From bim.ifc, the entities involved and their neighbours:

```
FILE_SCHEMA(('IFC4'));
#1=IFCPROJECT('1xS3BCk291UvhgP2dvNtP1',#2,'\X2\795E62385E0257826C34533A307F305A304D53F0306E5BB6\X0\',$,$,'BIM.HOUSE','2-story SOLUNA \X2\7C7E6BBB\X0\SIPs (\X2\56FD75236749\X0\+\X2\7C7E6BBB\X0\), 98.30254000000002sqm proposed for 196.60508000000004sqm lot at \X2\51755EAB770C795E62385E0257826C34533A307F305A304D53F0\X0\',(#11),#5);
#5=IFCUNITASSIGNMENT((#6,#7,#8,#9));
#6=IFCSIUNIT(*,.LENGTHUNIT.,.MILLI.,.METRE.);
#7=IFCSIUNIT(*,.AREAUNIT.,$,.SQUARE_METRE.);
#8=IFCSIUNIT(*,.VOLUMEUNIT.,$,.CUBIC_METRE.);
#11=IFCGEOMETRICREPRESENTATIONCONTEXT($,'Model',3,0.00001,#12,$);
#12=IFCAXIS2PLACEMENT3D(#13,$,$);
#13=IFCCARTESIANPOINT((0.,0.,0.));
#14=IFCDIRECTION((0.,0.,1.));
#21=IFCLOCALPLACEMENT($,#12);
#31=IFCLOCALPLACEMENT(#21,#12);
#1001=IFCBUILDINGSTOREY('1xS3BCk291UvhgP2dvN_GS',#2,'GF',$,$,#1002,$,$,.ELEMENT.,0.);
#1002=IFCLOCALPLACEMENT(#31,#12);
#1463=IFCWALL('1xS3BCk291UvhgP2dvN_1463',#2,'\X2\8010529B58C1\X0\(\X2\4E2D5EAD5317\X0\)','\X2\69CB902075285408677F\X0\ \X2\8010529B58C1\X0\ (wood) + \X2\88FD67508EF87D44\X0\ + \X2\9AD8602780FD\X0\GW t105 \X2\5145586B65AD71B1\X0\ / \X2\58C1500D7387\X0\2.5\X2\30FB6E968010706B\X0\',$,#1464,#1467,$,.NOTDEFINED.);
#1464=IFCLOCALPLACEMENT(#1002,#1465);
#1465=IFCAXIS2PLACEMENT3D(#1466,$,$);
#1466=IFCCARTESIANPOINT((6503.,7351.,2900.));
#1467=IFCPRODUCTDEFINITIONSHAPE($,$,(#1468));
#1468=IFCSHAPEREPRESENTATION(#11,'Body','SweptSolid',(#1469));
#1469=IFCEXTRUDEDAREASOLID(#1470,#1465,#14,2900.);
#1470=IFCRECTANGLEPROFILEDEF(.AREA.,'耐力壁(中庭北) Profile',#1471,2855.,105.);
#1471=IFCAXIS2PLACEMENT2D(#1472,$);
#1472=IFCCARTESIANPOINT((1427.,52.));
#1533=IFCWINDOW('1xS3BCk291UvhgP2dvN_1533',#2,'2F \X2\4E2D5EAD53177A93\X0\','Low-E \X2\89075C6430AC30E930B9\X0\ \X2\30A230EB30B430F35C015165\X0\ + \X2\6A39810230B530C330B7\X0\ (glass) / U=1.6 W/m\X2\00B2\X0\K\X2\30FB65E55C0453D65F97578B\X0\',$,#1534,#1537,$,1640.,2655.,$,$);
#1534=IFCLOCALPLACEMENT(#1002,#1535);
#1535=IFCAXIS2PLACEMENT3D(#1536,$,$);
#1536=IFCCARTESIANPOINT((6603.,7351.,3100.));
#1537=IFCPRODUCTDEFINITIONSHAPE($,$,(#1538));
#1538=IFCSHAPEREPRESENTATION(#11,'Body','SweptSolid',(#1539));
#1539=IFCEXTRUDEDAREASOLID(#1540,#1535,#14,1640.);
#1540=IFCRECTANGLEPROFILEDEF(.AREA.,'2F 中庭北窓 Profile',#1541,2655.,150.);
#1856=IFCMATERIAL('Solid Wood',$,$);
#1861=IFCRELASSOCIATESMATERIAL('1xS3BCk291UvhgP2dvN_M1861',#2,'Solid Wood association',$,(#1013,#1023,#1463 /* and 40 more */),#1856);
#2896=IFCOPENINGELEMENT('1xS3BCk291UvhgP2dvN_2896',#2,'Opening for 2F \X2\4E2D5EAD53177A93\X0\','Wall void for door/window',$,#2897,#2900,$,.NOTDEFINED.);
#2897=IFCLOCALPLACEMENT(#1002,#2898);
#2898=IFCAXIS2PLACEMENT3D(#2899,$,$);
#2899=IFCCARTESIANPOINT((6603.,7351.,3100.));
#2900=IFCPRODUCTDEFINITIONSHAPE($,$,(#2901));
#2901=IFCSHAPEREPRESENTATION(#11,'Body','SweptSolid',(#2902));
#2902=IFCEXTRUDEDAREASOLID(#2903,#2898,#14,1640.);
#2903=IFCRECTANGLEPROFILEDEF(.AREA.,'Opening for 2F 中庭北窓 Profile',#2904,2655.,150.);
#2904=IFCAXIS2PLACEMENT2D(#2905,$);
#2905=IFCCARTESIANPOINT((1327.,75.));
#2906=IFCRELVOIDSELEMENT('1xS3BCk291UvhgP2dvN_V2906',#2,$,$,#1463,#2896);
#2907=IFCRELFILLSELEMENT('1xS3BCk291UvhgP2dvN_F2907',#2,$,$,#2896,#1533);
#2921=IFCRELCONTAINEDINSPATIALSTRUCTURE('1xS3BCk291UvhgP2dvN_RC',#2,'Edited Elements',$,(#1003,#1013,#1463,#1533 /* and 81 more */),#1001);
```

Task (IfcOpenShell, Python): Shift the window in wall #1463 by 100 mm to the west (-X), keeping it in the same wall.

```python
import ifcopenshell
import ifcopenshell.api.geometry
import ifcopenshell.util.placement
import ifcopenshell.util.unit

model = ifcopenshell.open("bim.ifc")
unit_scale = ifcopenshell.util.unit.calculate_unit_scale(model)

window = model.by_id(1533)
opening = window.FillsVoids[0].RelatingOpeningElement
wall = opening.VoidsElements[0].RelatingBuildingElement

wall_matrix = ifcopenshell.util.placement.get_local_placement(wall.ObjectPlacement)
shift = wall_matrix[:3, 0] * -0.1 / unit_scale
before = ifcopenshell.util.placement.get_local_placement(window.ObjectPlacement)[:3, 3].copy()

# The window is not placed relative to its opening, so move both.
for product in (opening, window):
    matrix = ifcopenshell.util.placement.get_local_placement(product.ObjectPlacement)
    matrix[:3, 3] += shift
    ifcopenshell.api.geometry.edit_object_placement(model, product=product, matrix=matrix, is_si=False)

after = ifcopenshell.util.placement.get_local_placement(window.ObjectPlacement)[:3, 3]
print("window moved by", (after - before).round(3) + 0.0)

model.write("bim-out.ifc")
```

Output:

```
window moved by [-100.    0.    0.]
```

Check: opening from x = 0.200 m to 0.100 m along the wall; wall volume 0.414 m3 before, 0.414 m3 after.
